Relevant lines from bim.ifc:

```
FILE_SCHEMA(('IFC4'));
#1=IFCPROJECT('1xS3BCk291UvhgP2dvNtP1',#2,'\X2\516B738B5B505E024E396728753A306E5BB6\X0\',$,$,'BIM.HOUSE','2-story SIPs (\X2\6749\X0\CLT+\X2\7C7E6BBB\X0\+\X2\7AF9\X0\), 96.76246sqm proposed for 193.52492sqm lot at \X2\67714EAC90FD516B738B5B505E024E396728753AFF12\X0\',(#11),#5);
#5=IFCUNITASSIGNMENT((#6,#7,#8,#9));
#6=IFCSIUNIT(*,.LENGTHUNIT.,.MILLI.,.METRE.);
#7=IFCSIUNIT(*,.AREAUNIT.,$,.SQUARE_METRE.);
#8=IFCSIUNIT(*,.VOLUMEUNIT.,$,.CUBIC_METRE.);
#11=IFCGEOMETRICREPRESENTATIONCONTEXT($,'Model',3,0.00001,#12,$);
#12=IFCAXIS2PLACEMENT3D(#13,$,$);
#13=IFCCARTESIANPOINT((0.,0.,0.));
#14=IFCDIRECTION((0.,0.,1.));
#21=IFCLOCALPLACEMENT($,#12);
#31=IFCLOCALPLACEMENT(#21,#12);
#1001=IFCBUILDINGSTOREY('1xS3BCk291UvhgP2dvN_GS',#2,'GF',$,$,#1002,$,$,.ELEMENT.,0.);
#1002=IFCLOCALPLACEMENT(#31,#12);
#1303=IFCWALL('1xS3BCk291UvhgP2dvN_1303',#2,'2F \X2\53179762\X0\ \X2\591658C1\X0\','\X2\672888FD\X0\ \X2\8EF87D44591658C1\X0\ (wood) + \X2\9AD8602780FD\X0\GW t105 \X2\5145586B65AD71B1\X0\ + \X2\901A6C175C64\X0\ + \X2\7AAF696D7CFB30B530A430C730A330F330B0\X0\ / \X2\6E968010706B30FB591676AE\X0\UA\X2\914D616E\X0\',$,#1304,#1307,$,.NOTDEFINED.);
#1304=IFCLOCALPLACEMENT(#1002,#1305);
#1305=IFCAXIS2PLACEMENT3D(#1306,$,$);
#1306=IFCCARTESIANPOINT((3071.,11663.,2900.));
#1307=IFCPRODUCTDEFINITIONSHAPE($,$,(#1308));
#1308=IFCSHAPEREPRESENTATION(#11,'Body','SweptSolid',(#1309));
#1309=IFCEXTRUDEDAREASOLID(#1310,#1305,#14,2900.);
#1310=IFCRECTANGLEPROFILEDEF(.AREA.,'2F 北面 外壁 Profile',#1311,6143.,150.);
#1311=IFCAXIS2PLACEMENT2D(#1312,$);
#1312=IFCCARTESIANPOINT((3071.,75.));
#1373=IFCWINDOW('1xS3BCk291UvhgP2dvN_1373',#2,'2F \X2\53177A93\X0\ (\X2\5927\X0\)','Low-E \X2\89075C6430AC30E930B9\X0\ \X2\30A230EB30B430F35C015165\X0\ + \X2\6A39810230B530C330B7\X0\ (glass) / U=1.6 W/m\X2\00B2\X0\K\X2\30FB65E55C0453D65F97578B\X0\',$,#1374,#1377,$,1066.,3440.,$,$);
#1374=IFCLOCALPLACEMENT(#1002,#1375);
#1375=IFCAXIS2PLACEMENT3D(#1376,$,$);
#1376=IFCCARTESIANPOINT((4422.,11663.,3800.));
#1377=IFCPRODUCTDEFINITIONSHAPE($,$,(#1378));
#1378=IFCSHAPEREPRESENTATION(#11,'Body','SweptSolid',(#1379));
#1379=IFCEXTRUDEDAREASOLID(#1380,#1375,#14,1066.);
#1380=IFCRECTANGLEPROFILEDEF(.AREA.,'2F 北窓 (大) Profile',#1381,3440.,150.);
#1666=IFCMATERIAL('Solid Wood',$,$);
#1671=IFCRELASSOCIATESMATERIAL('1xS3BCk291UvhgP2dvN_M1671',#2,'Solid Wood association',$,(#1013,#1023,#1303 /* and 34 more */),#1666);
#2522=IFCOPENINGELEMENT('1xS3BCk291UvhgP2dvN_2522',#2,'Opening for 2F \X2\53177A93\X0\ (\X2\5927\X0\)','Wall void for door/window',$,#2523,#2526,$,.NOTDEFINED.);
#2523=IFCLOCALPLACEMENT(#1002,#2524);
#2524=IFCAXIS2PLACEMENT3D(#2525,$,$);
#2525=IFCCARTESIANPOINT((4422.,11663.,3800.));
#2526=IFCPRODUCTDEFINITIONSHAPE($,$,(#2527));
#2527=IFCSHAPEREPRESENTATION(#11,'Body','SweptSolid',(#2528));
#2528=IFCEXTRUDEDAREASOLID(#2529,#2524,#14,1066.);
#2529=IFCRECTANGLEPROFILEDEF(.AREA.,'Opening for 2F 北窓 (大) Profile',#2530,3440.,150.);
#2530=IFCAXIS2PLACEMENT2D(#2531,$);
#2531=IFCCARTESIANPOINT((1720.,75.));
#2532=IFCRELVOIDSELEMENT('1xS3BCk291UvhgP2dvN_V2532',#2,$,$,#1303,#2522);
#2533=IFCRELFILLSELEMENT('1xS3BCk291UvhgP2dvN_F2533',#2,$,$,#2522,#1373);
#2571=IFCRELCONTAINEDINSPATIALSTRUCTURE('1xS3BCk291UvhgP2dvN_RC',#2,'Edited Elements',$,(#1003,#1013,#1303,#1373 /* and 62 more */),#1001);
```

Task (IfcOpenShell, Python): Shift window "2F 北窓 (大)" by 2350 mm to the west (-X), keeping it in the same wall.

```python
import ifcopenshell
import ifcopenshell.api.geometry
import ifcopenshell.util.placement

model = ifcopenshell.open("bim.ifc")

window = model.by_guid("1xS3BCk291UvhgP2dvN_1373")
opening = window.FillsVoids[0].RelatingOpeningElement
wall = opening.VoidsElements[0].RelatingBuildingElement

wall_matrix = ifcopenshell.util.placement.get_local_placement(wall.ObjectPlacement)
shift = wall_matrix[:3, 0] * -2350.0
before = ifcopenshell.util.placement.get_local_placement(window.ObjectPlacement)[:3, 3].copy()

# The window is not placed relative to its opening, so move both.
for product in (opening, window):
    matrix = ifcopenshell.util.placement.get_local_placement(product.ObjectPlacement)
    matrix[:3, 3] += shift
    ifcopenshell.api.geometry.edit_object_placement(model, product=product, matrix=matrix, is_si=False)

after = ifcopenshell.util.placement.get_local_placement(window.ObjectPlacement)[:3, 3]
print("window moved by", (after - before).round(3) + 0.0)

model.write("bim_edited.ifc")
```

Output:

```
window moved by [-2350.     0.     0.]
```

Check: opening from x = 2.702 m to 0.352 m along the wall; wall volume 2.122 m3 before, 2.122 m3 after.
